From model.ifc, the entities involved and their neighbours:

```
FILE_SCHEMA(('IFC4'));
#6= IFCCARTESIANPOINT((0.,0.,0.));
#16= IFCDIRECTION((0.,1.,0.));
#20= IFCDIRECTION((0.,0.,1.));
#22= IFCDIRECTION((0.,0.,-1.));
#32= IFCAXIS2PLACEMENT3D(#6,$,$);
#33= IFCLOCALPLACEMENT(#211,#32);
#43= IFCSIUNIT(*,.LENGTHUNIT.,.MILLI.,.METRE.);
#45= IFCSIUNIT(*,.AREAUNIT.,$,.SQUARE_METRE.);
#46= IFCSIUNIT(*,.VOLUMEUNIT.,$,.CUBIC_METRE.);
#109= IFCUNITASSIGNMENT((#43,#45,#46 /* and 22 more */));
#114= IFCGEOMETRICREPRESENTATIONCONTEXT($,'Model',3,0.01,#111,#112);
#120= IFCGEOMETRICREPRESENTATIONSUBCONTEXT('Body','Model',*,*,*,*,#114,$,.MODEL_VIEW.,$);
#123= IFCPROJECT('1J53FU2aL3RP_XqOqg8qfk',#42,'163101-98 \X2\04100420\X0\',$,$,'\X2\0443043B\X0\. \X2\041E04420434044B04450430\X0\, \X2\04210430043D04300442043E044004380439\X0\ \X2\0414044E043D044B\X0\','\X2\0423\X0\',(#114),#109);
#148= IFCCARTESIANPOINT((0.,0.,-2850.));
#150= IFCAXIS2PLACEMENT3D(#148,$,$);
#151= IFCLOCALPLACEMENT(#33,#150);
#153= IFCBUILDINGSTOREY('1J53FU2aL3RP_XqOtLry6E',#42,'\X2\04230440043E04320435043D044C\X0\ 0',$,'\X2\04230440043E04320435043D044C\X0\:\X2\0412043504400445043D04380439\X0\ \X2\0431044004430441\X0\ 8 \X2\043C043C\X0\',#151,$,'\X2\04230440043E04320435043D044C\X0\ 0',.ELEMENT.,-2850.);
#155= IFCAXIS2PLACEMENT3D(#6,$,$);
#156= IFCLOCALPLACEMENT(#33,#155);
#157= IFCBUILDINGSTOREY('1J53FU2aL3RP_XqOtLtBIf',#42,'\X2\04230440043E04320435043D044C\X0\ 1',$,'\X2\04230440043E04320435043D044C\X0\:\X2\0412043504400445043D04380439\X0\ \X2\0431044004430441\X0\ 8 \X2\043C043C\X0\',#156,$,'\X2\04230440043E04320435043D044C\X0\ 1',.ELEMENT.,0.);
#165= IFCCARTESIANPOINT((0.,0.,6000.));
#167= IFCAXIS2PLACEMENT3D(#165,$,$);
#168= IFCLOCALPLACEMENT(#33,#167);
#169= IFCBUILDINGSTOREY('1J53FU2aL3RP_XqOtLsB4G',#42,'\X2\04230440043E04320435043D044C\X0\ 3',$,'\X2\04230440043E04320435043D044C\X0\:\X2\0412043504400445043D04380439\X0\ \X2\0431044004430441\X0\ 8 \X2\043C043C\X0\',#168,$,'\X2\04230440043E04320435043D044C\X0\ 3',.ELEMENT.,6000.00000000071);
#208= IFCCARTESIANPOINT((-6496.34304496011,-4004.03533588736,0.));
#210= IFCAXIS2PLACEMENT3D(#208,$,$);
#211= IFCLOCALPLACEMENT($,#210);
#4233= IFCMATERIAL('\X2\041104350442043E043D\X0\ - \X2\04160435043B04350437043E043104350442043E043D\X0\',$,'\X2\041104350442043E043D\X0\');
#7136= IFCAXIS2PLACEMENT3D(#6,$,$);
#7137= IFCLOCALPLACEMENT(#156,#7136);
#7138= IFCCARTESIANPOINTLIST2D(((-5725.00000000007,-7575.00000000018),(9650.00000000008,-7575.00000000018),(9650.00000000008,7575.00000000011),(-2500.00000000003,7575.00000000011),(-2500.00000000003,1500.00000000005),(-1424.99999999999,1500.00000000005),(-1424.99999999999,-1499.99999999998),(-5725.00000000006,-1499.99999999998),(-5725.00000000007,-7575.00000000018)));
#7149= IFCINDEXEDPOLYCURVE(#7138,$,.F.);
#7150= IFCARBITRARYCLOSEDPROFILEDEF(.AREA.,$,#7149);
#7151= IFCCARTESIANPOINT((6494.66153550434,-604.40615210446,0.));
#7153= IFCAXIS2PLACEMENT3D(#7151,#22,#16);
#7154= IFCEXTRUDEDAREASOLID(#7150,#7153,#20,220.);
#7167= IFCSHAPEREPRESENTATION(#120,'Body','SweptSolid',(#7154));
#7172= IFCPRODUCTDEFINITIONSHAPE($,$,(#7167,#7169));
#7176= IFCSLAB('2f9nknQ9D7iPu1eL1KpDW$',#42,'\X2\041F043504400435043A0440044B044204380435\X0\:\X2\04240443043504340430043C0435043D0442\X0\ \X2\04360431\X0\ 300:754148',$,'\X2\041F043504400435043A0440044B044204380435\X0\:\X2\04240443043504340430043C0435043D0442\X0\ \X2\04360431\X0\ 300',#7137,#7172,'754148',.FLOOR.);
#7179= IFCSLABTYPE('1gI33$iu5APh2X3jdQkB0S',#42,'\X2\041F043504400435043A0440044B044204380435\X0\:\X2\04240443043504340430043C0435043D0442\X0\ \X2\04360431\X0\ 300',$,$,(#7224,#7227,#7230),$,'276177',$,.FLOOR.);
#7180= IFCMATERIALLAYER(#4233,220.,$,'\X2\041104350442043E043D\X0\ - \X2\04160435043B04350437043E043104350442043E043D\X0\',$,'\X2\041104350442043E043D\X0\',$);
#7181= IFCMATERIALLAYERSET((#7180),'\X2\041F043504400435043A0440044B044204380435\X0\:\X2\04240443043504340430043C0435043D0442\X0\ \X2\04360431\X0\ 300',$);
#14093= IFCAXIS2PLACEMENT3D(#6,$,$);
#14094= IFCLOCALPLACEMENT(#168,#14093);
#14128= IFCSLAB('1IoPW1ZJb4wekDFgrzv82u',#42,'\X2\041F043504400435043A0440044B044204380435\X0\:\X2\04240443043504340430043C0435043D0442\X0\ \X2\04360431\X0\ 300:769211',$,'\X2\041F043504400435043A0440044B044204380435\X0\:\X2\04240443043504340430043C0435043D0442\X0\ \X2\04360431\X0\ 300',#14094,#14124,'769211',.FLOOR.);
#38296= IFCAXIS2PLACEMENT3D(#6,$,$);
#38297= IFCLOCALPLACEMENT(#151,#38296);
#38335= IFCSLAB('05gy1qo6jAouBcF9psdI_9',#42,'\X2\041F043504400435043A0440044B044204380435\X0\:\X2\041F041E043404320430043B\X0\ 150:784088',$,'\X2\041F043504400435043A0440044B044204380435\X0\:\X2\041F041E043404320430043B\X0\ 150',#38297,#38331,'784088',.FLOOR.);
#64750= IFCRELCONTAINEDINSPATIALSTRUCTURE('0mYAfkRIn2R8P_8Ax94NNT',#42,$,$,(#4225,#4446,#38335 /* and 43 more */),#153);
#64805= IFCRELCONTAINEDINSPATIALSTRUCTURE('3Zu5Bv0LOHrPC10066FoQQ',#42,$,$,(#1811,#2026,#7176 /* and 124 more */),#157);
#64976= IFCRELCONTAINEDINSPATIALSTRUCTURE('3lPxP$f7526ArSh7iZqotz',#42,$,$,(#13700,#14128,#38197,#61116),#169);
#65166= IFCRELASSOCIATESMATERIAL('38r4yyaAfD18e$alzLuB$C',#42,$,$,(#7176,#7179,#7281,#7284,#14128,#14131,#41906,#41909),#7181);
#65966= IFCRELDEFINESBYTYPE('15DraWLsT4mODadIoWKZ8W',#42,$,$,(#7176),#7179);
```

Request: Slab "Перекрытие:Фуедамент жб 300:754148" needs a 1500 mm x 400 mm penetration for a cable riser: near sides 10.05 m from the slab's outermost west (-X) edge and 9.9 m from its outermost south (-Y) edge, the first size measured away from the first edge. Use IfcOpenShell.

```python
import numpy as np
import ifcopenshell
import ifcopenshell.api.feature
import ifcopenshell.api.geometry
import ifcopenshell.api.root
import ifcopenshell.geom
import ifcopenshell.util.placement
import ifcopenshell.util.representation
import ifcopenshell.util.shape
import ifcopenshell.util.unit

model = ifcopenshell.open("model.ifc")
unit_scale = ifcopenshell.util.unit.calculate_unit_scale(model)
settings = ifcopenshell.geom.settings()


def volume(element):
    """Net volume in cubic metres, openings subtracted."""
    shape = ifcopenshell.geom.create_shape(settings, element)
    return ifcopenshell.util.shape.get_volume(shape.geometry)


slab = model.by_guid("2f9nknQ9D7iPu1eL1KpDW$")
before = volume(slab)

# Extent in the slab's own axes, in metres. The edges named are its -X and -Y sides.
slab_shape = ifcopenshell.geom.create_shape(settings, slab)
vertices = ifcopenshell.util.shape.get_vertices(slab_shape.geometry)
x_min, y_min, bottom = vertices.min(axis=0)
top = vertices[:, 2].max()

opening = ifcopenshell.api.root.create_entity(model, ifc_class="IfcOpeningElement", name="Cable riser opening", predefined_type="OPENING")
context = ifcopenshell.util.representation.get_context(model, "Model", "Body", "MODEL_VIEW")
width, depth = 1.5, 0.4
outline = [(0.0, 0.0), (width, 0.0), (width, depth), (0.0, depth), (0.0, 0.0)]
# Overshoot both faces by 50 mm so the cut is clean.
shape = ifcopenshell.api.geometry.add_slab_representation(
    model, context=context, depth=top - bottom + 0.1, polyline=outline
)
ifcopenshell.api.geometry.assign_representation(model, product=opening, representation=shape)

matrix = ifcopenshell.util.placement.get_local_placement(slab.ObjectPlacement)
matrix[:, 3] = matrix @ np.append(np.array([x_min + 10.05, y_min + 9.9, bottom - 0.05]) / unit_scale, 1.0)
ifcopenshell.api.geometry.edit_object_placement(model, product=opening, matrix=matrix, is_si=False)
ifcopenshell.api.feature.add_feature(model, feature=opening, element=slab)

after = volume(slab)

print(f"slab volume {before:.3f} -> {after:.3f} m3")

model.write("model_updated.ifc")
```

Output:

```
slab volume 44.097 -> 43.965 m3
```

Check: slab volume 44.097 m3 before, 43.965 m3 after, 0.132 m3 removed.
